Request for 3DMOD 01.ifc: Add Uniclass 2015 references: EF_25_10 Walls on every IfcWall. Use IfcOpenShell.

First a look at what the model holds.

```python
import ifcopenshell

model = ifcopenshell.open("3DMOD 01.ifc")
print(model.schema)
print("classifications:", [c.Name for c in model.by_type("IfcClassification")])
for ifc_class in ("IfcDoor", "IfcRoof", "IfcStair", "IfcWall", "IfcWindow"):
    print(ifc_class, len(model.by_type(ifc_class)))
```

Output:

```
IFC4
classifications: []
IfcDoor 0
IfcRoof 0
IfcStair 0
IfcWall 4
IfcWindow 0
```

```python
import ifcopenshell
import ifcopenshell.api.classification

model = ifcopenshell.open("3DMOD 01.ifc")

system = ifcopenshell.api.classification.add_classification(model, classification="Uniclass 2015")

codes = {
    "IfcWall": ("EF_25_10", "Walls"),
}
for ifc_class, (code, name) in codes.items():
    products = model.by_type(ifc_class)
    ifcopenshell.api.classification.add_reference(
        model, products=products, classification=system, identification=code, name=name
    )
    print(code, len(products))

model.write("3DMOD 01_rev.ifc")
```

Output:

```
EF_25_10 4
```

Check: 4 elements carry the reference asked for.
